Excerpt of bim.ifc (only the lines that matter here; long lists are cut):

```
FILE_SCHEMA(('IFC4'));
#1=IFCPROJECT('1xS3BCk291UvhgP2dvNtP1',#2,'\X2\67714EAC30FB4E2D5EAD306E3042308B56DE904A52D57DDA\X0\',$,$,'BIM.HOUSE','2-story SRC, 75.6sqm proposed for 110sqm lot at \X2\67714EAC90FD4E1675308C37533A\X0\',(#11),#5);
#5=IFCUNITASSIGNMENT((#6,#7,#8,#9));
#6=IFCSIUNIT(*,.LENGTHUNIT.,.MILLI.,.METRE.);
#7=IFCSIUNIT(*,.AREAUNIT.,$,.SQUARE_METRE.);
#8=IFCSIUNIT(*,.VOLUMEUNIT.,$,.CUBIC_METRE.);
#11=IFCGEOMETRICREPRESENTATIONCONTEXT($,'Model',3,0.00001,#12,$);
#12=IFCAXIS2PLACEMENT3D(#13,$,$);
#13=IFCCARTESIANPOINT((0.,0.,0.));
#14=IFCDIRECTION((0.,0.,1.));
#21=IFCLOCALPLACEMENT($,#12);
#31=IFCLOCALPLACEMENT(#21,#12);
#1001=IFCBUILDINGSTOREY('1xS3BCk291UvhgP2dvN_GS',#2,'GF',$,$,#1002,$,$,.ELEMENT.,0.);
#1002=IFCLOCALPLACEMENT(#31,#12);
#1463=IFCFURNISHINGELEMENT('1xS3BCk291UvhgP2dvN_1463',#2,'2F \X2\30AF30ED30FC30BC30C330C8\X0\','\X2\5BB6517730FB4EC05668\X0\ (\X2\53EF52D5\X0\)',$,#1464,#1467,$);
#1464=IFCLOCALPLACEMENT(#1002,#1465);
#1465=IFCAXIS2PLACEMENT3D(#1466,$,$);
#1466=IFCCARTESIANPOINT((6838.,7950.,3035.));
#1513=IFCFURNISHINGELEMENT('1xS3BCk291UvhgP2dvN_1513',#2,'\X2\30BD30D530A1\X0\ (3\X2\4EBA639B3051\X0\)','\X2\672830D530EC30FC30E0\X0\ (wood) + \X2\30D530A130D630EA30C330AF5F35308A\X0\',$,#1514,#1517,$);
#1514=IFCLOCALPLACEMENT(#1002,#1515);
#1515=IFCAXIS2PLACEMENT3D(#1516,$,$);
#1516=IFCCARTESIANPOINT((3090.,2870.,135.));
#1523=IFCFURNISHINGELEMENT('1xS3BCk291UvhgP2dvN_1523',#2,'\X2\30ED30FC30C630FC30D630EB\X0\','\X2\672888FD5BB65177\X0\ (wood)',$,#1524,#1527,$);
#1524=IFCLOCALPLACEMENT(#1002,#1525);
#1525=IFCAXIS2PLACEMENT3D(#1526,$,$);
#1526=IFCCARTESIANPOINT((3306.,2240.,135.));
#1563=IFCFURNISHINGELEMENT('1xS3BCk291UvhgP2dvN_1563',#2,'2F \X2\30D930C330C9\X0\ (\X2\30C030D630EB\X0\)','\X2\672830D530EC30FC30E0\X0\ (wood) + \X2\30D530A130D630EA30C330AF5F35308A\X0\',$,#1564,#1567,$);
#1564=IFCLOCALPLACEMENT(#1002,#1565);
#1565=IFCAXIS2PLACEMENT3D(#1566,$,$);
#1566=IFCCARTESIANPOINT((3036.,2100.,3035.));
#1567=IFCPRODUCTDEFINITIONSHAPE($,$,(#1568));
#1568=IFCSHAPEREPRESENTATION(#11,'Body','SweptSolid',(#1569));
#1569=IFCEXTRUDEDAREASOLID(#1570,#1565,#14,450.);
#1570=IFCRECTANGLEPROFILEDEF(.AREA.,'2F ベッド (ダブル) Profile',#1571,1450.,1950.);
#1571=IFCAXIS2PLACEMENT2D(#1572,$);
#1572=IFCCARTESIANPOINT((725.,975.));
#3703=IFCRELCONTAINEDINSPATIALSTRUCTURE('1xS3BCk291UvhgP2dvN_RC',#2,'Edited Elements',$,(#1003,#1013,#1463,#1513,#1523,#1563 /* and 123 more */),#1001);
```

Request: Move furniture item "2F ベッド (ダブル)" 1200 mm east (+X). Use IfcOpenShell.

```python
import ifcopenshell
import ifcopenshell.api.geometry
import ifcopenshell.util.placement
import ifcopenshell.util.unit

model = ifcopenshell.open("bim.ifc")
unit_scale = ifcopenshell.util.unit.calculate_unit_scale(model)

item = model.by_guid("1xS3BCk291UvhgP2dvN_1563")
matrix = ifcopenshell.util.placement.get_local_placement(item.ObjectPlacement)
matrix[0, 3] += 1.2 / unit_scale
ifcopenshell.api.geometry.edit_object_placement(model, product=item, matrix=matrix, is_si=False)

print(ifcopenshell.util.placement.get_local_placement(item.ObjectPlacement).round(3) + 0.0)

model.write("bim_edited.ifc")
```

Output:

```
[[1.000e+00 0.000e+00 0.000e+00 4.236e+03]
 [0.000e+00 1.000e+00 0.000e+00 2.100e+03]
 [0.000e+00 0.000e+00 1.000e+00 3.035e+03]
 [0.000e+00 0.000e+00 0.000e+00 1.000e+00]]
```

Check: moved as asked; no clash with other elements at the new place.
